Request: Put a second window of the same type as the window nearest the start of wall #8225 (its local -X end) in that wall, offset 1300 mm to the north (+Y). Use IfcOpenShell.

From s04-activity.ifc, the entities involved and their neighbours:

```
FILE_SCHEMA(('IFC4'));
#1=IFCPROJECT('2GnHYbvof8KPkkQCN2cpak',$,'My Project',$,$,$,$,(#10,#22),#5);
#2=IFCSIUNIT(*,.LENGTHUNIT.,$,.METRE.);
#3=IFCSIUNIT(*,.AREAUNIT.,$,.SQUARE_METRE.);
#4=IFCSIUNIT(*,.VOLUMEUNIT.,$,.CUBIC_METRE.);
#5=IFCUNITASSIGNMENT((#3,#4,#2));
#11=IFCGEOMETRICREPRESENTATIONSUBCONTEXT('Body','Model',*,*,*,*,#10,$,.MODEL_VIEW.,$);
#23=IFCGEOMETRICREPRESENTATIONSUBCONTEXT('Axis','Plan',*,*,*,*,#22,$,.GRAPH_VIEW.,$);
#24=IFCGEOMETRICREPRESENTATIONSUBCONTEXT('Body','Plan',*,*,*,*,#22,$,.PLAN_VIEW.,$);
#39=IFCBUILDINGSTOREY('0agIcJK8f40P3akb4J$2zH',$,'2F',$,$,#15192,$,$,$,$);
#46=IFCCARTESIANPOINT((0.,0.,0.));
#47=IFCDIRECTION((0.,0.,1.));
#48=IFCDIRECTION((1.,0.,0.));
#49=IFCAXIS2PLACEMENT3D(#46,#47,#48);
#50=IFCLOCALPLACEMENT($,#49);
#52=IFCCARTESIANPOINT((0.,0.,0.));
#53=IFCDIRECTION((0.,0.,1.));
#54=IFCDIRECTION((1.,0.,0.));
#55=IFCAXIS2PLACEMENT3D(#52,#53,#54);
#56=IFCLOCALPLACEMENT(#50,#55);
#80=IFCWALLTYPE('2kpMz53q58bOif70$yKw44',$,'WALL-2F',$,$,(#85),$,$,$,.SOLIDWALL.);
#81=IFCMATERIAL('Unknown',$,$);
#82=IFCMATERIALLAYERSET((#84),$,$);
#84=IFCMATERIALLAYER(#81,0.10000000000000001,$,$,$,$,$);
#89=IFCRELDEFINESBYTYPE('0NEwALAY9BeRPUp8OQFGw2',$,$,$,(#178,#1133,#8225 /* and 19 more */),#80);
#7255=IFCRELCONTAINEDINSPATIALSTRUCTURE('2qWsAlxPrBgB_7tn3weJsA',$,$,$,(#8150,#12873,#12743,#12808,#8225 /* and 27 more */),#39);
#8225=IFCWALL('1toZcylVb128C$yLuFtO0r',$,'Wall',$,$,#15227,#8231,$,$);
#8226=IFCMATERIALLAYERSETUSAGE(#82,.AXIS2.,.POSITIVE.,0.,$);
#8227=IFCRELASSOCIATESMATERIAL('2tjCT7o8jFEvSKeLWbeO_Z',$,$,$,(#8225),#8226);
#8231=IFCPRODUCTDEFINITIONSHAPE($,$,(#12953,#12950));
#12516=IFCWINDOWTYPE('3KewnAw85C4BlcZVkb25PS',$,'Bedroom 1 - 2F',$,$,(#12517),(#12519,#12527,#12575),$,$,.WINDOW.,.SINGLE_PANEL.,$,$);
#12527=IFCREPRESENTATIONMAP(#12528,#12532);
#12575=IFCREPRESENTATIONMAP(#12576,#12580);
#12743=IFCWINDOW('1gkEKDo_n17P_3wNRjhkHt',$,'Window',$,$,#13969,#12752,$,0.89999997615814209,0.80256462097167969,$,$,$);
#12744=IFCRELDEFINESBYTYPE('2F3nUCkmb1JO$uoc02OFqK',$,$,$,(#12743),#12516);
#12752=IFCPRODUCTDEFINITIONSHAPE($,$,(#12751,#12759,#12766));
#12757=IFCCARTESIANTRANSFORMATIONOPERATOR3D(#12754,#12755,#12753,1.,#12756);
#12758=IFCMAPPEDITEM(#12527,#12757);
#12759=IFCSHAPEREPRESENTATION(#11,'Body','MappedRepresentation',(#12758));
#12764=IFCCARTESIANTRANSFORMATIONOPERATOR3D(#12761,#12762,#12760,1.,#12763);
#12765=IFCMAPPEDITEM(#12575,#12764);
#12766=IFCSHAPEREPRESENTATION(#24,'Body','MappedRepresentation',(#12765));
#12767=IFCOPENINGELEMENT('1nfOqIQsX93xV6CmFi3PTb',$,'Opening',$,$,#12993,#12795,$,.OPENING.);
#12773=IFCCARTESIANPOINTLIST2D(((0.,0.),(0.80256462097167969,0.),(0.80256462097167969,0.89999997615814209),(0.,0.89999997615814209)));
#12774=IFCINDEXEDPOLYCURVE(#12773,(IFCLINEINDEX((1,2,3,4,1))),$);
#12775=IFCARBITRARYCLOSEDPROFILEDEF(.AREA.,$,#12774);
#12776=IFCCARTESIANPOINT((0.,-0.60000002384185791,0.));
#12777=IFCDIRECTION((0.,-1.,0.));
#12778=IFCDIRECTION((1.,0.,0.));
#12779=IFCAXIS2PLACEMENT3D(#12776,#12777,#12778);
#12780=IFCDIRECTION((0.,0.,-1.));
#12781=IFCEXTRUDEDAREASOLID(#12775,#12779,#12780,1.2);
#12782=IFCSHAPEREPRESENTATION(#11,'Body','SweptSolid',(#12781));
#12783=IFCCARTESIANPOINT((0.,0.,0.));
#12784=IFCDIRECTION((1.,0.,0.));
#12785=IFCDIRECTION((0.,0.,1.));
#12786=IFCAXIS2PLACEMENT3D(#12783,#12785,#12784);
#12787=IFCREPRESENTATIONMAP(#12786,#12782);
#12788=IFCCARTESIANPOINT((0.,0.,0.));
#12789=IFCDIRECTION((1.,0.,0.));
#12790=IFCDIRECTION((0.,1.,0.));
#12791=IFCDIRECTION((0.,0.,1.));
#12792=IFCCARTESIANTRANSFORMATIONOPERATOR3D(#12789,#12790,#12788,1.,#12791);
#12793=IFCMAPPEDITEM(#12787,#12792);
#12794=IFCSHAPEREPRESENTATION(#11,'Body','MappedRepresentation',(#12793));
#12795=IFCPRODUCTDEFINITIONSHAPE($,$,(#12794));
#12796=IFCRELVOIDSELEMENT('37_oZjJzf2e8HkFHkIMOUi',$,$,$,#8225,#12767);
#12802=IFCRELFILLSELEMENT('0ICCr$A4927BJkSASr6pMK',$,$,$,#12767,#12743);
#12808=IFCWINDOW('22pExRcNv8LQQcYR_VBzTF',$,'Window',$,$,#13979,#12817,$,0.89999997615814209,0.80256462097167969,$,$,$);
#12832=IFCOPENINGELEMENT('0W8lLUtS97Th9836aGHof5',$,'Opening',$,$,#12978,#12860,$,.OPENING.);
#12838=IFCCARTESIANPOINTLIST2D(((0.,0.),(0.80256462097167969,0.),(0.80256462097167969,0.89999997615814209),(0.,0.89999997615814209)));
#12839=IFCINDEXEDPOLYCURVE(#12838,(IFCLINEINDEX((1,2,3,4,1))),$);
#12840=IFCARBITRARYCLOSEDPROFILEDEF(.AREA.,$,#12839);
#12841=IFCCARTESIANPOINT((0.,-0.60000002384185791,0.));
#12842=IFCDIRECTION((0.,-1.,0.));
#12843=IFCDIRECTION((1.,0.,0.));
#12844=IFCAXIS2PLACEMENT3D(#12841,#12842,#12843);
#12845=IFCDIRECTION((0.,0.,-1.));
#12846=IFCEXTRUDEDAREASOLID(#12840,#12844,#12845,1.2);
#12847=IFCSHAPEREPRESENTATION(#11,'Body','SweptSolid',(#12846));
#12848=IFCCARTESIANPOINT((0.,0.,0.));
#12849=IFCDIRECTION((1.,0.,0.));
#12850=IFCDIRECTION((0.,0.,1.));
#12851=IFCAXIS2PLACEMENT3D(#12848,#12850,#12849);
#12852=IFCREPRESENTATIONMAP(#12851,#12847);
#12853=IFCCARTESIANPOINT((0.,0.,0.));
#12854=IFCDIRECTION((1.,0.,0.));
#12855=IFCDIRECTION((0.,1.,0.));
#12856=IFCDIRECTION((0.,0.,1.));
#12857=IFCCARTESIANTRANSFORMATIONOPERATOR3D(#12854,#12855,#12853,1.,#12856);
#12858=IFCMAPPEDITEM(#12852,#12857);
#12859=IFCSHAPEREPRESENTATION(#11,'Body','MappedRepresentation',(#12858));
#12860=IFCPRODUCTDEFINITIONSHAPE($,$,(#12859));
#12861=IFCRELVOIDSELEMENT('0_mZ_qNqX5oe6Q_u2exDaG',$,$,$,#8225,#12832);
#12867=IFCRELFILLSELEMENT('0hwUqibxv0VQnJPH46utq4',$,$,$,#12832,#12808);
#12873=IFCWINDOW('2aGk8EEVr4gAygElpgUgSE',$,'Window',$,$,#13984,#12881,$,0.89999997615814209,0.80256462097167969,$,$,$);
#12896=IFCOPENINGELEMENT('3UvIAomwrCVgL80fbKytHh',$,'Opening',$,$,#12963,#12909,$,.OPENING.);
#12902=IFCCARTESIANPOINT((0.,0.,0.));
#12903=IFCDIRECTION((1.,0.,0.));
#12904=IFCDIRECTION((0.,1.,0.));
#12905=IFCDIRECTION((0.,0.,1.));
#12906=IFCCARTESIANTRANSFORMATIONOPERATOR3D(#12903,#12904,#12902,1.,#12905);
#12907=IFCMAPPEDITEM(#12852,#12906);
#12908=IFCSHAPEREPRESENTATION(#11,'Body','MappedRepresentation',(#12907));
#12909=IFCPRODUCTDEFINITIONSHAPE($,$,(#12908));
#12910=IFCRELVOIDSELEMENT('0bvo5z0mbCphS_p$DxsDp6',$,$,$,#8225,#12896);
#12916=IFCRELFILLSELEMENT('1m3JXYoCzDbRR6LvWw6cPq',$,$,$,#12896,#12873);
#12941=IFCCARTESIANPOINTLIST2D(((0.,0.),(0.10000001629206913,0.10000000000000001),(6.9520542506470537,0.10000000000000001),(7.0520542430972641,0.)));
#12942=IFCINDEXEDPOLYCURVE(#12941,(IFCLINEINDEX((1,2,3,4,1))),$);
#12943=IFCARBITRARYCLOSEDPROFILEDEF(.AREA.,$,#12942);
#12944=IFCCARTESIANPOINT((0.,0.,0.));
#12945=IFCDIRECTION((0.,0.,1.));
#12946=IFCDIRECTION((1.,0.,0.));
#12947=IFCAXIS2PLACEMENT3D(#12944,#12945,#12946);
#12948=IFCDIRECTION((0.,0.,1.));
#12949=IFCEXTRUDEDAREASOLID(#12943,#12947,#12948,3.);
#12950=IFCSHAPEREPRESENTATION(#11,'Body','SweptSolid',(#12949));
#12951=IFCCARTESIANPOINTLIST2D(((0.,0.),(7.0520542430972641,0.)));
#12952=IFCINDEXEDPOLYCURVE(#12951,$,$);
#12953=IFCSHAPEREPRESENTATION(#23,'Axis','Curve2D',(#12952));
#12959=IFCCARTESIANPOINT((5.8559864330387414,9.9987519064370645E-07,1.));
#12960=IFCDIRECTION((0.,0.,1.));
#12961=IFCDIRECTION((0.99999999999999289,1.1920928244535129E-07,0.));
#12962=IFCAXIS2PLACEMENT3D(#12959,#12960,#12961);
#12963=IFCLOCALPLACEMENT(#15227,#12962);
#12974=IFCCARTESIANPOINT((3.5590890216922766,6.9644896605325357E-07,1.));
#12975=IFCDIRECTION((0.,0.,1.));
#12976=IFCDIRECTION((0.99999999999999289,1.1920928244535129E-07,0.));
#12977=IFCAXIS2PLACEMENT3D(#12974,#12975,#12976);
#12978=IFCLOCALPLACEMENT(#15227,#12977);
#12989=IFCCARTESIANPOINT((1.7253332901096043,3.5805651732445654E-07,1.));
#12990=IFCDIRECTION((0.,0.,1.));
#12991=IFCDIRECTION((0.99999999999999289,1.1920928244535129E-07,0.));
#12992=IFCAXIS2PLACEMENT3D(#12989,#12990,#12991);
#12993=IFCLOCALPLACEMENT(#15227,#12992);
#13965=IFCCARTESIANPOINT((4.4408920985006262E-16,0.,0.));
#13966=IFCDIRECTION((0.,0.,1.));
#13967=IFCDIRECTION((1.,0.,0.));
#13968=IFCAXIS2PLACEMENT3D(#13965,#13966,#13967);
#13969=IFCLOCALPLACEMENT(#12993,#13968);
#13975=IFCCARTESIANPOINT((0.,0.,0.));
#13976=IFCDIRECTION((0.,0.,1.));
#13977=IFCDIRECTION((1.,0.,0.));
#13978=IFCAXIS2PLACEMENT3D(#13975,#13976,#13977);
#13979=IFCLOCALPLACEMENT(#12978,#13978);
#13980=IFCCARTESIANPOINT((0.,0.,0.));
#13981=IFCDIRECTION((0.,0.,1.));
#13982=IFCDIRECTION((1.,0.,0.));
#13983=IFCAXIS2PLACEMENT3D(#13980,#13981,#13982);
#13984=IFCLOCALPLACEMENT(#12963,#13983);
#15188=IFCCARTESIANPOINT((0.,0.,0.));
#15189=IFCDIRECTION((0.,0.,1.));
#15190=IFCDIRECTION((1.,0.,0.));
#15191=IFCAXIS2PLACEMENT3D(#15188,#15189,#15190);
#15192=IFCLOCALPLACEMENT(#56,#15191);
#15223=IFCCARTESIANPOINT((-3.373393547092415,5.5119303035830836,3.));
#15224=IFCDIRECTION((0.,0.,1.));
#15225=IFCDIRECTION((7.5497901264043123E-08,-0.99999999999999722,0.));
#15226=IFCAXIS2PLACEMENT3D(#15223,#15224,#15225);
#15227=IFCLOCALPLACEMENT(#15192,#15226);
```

```python
import ifcopenshell
import ifcopenshell.api.feature
import ifcopenshell.api.geometry
import ifcopenshell.api.root
import ifcopenshell.geom
import ifcopenshell.util.element
import ifcopenshell.util.placement
import ifcopenshell.util.shape
import ifcopenshell.util.unit

model = ifcopenshell.open("s04-activity.ifc")
unit_scale = ifcopenshell.util.unit.calculate_unit_scale(model)
settings = ifcopenshell.geom.settings()


def volume(element):
    """Net volume in cubic metres, openings subtracted."""
    shape = ifcopenshell.geom.create_shape(settings, element)
    return ifcopenshell.util.shape.get_volume(shape.geometry)


window = model.by_id(12743)
opening = window.FillsVoids[0].RelatingOpeningElement
wall = opening.VoidsElements[0].RelatingBuildingElement
before = volume(wall)
shift = ifcopenshell.util.placement.get_local_placement(wall.ObjectPlacement)[:3, 0] * -1.3 / unit_scale

# copy_class copies the void relationship, type, container and properties, but no geometry.
new_opening = ifcopenshell.api.root.copy_class(model, product=opening)
new_opening.Representation = ifcopenshell.util.element.copy_deep(
    model, opening.Representation, exclude=["IfcGeometricRepresentationContext", "IfcRepresentationMap"]
)
new_window = ifcopenshell.api.root.copy_class(model, product=window)
new_window.Representation = ifcopenshell.util.element.copy_deep(
    model, window.Representation, exclude=["IfcGeometricRepresentationContext", "IfcRepresentationMap"]
)
ifcopenshell.api.feature.add_filling(model, opening=new_opening, element=new_window)

for old, new in ((opening, new_opening), (window, new_window)):
    matrix = ifcopenshell.util.placement.get_local_placement(old.ObjectPlacement)
    matrix[:3, 3] += shift
    ifcopenshell.api.geometry.edit_object_placement(model, product=new, matrix=matrix, is_si=False)

after = volume(wall)

print(f"wall volume {before:.3f} -> {after:.3f} m3")

model.write("s04-activity-out.ifc")
```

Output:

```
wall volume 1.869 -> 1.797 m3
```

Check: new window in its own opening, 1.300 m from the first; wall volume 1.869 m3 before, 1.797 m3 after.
